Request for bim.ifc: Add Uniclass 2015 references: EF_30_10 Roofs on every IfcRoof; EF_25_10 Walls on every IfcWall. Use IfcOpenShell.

First a look at what the model holds.

```python
import ifcopenshell

model = ifcopenshell.open("bim.ifc")
print(model.schema)
print("classifications:", [c.Name for c in model.by_type("IfcClassification")])
for ifc_class in ("IfcDoor", "IfcRoof", "IfcStair", "IfcWall", "IfcWindow"):
    print(ifc_class, len(model.by_type(ifc_class)))
```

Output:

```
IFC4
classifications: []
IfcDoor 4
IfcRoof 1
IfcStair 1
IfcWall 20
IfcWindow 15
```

```python
import ifcopenshell
import ifcopenshell.api.classification

model = ifcopenshell.open("bim.ifc")

system = ifcopenshell.api.classification.add_classification(model, classification="Uniclass 2015")

codes = {
    "IfcRoof": ("EF_30_10", "Roofs"),
    "IfcWall": ("EF_25_10", "Walls"),
}
for ifc_class, (code, name) in codes.items():
    products = model.by_type(ifc_class)
    ifcopenshell.api.classification.add_reference(
        model, products=products, classification=system, identification=code, name=name
    )
    print(code, len(products))

model.write("bim_rev.ifc")
```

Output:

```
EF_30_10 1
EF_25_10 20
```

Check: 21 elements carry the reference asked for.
